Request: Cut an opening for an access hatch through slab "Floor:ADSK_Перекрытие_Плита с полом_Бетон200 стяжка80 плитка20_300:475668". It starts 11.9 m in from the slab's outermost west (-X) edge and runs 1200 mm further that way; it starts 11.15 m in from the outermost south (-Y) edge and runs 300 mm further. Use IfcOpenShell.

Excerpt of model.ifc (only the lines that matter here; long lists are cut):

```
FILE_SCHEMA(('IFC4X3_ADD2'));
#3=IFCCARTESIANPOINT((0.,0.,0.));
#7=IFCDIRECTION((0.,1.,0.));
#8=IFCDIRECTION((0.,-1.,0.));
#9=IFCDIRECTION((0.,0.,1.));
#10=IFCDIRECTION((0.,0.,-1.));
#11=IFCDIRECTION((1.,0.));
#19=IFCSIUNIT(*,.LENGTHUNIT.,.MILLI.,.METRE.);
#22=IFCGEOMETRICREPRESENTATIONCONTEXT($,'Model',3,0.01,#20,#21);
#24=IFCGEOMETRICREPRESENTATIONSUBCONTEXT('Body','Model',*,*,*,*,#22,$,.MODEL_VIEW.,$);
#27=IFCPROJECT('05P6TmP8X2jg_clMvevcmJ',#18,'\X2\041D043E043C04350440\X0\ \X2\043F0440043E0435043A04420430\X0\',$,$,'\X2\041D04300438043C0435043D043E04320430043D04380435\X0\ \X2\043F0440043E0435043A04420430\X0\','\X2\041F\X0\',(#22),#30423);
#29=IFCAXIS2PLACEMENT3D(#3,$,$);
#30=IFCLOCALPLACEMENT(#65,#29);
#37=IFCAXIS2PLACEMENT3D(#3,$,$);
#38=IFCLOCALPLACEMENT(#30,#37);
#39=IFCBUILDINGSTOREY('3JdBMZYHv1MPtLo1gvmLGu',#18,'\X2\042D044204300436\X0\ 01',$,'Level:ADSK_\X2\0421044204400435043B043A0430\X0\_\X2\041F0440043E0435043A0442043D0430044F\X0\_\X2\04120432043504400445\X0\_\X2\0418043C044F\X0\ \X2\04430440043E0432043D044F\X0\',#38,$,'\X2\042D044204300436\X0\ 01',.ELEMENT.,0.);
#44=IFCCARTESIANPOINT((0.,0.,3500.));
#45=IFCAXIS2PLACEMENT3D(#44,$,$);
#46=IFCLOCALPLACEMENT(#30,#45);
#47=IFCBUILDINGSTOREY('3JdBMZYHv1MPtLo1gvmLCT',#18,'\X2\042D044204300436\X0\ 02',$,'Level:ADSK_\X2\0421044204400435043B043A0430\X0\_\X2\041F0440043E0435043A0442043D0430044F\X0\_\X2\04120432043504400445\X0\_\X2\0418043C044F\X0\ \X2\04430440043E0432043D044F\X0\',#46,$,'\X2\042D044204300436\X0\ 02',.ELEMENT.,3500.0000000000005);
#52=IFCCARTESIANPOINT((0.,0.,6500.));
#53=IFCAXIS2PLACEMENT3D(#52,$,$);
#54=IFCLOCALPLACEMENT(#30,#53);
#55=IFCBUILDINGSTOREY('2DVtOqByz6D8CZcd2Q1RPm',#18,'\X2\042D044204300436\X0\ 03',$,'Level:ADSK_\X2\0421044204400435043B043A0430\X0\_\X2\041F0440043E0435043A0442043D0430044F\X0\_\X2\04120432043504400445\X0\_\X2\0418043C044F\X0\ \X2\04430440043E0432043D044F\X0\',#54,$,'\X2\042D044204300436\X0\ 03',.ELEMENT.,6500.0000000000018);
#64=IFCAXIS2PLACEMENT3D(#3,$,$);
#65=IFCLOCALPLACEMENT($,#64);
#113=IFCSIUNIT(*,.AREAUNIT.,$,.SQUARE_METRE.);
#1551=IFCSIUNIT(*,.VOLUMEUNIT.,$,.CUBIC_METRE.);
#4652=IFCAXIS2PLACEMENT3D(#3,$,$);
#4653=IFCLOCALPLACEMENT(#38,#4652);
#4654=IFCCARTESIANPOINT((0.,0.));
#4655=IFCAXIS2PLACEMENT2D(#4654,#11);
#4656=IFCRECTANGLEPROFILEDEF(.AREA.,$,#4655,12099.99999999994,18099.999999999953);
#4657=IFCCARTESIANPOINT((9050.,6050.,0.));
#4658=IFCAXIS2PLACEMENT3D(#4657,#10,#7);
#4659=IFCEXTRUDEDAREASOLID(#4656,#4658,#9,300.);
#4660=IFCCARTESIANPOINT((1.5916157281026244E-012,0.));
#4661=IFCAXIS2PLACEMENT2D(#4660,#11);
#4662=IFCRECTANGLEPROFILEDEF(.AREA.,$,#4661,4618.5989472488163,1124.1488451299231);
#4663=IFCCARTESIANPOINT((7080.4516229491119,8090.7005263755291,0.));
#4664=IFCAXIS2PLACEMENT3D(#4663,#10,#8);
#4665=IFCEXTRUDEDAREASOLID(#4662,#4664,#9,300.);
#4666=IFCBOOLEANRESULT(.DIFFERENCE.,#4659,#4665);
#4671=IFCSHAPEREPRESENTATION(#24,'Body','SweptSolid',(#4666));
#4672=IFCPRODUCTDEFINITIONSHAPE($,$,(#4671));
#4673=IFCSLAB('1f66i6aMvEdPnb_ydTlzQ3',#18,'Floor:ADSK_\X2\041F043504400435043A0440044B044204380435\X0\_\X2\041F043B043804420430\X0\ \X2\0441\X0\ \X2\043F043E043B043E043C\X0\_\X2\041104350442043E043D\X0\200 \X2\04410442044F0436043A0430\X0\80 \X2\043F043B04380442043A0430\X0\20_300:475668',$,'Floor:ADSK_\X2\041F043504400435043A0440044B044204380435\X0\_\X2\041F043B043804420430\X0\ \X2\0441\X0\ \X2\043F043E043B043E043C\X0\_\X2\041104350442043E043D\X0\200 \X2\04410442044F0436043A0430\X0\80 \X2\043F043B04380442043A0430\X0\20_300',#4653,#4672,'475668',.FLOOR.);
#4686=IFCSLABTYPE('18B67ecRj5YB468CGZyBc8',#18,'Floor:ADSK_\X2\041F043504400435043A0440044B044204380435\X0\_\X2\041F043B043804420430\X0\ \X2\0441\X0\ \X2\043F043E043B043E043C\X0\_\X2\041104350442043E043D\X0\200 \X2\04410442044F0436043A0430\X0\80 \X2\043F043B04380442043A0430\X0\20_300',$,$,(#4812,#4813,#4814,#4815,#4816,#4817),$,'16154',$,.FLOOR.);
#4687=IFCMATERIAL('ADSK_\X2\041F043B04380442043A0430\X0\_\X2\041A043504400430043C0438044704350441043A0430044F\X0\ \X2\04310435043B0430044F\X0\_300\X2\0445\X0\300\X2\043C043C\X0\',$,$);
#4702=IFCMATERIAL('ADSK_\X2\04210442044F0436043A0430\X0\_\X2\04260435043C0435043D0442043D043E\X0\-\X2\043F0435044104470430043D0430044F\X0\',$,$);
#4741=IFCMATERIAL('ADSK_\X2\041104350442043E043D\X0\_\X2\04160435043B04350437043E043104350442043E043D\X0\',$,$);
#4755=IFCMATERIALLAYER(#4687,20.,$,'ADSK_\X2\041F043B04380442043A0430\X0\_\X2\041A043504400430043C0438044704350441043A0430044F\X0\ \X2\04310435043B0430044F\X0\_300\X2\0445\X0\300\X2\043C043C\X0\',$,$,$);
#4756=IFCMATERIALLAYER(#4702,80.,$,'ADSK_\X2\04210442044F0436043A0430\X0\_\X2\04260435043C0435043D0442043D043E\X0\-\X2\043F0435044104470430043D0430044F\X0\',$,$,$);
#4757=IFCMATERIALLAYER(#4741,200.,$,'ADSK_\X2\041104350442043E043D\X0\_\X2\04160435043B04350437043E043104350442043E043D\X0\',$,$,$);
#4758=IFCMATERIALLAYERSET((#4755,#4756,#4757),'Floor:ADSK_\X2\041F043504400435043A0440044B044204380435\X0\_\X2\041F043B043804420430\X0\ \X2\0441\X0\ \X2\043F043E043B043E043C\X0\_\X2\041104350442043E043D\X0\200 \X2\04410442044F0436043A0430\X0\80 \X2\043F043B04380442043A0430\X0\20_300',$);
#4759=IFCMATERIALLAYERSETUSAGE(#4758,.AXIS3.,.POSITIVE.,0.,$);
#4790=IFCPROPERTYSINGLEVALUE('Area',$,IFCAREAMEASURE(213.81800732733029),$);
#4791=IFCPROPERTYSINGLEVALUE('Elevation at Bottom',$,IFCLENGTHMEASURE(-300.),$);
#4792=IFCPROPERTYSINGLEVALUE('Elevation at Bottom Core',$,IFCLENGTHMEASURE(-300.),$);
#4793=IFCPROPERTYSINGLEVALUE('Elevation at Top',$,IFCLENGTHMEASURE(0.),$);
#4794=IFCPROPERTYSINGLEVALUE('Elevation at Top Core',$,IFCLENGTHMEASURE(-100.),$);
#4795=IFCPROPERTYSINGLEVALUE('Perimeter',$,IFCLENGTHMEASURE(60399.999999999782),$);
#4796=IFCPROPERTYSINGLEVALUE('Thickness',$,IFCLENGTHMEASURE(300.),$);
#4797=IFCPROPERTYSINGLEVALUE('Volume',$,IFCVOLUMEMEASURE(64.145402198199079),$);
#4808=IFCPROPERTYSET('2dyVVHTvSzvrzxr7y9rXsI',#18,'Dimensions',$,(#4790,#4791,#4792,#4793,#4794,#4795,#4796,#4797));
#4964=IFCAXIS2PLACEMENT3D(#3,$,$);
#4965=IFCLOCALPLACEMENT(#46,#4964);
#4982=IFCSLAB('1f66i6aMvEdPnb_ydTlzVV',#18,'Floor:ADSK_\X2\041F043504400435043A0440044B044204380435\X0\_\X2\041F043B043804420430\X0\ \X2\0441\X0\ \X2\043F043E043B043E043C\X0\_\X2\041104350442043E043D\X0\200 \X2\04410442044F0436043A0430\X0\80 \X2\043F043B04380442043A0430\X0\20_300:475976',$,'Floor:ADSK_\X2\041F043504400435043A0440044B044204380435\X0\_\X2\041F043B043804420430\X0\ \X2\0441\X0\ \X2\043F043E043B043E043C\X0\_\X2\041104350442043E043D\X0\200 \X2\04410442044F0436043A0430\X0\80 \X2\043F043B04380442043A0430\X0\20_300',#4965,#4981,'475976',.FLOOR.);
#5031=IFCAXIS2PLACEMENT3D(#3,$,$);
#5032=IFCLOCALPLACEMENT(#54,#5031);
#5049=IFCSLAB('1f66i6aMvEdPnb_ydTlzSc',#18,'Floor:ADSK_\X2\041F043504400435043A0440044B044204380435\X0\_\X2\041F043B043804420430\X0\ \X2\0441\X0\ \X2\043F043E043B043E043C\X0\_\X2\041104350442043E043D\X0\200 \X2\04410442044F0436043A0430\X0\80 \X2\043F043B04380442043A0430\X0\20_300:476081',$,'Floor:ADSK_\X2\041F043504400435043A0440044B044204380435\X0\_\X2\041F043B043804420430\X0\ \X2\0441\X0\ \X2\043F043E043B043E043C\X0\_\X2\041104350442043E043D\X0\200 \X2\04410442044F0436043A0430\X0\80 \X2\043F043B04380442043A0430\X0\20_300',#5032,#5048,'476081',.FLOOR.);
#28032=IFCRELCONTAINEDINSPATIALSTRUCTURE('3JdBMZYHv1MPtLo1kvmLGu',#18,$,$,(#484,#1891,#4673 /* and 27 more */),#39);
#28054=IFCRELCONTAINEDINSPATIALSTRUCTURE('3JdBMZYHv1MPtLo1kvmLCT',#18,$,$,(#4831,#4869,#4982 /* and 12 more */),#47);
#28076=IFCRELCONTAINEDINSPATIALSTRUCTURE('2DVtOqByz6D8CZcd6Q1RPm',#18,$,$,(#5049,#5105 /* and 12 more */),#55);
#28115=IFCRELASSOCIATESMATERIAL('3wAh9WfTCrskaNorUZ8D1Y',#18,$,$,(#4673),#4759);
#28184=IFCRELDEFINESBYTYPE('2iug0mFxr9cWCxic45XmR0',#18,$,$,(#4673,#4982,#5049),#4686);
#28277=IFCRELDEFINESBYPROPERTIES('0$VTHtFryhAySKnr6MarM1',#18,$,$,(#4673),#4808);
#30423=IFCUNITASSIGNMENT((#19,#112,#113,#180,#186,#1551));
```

```python
import numpy as np
import ifcopenshell
import ifcopenshell.api.feature
import ifcopenshell.api.geometry
import ifcopenshell.api.pset
import ifcopenshell.api.root
import ifcopenshell.geom
import ifcopenshell.util.element
import ifcopenshell.util.placement
import ifcopenshell.util.representation
import ifcopenshell.util.shape
import ifcopenshell.util.unit

model = ifcopenshell.open("model.ifc")
unit_scale = ifcopenshell.util.unit.calculate_unit_scale(model)
area_scale = ifcopenshell.util.unit.calculate_unit_scale(model, "AREAUNIT")
volume_scale = ifcopenshell.util.unit.calculate_unit_scale(model, "VOLUMEUNIT")
settings = ifcopenshell.geom.settings()


def volume(element):
    """Net volume in cubic metres, openings subtracted."""
    shape = ifcopenshell.geom.create_shape(settings, element)
    return ifcopenshell.util.shape.get_volume(shape.geometry)


slab = model.by_guid("1f66i6aMvEdPnb_ydTlzQ3")
before = volume(slab)

# Extent in the slab's own axes, in metres. The edges named are its -X and -Y sides.
slab_shape = ifcopenshell.geom.create_shape(settings, slab)
vertices = ifcopenshell.util.shape.get_vertices(slab_shape.geometry)
x_min, y_min, bottom = vertices.min(axis=0)
top = vertices[:, 2].max()

opening = ifcopenshell.api.root.create_entity(model, ifc_class="IfcOpeningElement", name="Access hatch opening", predefined_type="OPENING")
context = ifcopenshell.util.representation.get_context(model, "Model", "Body", "MODEL_VIEW")
width, depth = 1.2, 0.3
outline = [(0.0, 0.0), (width, 0.0), (width, depth), (0.0, depth), (0.0, 0.0)]
# Overshoot both faces by 50 mm so the cut is clean.
shape = ifcopenshell.api.geometry.add_slab_representation(
    model, context=context, depth=top - bottom + 0.1, polyline=outline
)
ifcopenshell.api.geometry.assign_representation(model, product=opening, representation=shape)

matrix = ifcopenshell.util.placement.get_local_placement(slab.ObjectPlacement)
matrix[:, 3] = matrix @ np.append(np.array([x_min + 11.9, y_min + 11.15, bottom - 0.05]) / unit_scale, 1.0)
ifcopenshell.api.geometry.edit_object_placement(model, product=opening, matrix=matrix, is_si=False)
ifcopenshell.api.feature.add_feature(model, feature=opening, element=slab)

after = volume(slab)

# Update the slab's stored quantities.
pset = model.by_id(ifcopenshell.util.element.get_pset(slab, "Dimensions", should_inherit=False)["id"])
ifcopenshell.api.pset.edit_pset(model, pset=pset, properties={
    "Area": model.create_entity("IfcAreaMeasure", after / (top - bottom) / area_scale),
    "Volume": model.create_entity("IfcVolumeMeasure", after / volume_scale),
})

print(f"slab volume {before:.3f} -> {after:.3f} m3")

model.write("model_edited.ifc")
```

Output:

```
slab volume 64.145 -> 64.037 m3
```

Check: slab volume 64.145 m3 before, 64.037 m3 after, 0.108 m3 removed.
